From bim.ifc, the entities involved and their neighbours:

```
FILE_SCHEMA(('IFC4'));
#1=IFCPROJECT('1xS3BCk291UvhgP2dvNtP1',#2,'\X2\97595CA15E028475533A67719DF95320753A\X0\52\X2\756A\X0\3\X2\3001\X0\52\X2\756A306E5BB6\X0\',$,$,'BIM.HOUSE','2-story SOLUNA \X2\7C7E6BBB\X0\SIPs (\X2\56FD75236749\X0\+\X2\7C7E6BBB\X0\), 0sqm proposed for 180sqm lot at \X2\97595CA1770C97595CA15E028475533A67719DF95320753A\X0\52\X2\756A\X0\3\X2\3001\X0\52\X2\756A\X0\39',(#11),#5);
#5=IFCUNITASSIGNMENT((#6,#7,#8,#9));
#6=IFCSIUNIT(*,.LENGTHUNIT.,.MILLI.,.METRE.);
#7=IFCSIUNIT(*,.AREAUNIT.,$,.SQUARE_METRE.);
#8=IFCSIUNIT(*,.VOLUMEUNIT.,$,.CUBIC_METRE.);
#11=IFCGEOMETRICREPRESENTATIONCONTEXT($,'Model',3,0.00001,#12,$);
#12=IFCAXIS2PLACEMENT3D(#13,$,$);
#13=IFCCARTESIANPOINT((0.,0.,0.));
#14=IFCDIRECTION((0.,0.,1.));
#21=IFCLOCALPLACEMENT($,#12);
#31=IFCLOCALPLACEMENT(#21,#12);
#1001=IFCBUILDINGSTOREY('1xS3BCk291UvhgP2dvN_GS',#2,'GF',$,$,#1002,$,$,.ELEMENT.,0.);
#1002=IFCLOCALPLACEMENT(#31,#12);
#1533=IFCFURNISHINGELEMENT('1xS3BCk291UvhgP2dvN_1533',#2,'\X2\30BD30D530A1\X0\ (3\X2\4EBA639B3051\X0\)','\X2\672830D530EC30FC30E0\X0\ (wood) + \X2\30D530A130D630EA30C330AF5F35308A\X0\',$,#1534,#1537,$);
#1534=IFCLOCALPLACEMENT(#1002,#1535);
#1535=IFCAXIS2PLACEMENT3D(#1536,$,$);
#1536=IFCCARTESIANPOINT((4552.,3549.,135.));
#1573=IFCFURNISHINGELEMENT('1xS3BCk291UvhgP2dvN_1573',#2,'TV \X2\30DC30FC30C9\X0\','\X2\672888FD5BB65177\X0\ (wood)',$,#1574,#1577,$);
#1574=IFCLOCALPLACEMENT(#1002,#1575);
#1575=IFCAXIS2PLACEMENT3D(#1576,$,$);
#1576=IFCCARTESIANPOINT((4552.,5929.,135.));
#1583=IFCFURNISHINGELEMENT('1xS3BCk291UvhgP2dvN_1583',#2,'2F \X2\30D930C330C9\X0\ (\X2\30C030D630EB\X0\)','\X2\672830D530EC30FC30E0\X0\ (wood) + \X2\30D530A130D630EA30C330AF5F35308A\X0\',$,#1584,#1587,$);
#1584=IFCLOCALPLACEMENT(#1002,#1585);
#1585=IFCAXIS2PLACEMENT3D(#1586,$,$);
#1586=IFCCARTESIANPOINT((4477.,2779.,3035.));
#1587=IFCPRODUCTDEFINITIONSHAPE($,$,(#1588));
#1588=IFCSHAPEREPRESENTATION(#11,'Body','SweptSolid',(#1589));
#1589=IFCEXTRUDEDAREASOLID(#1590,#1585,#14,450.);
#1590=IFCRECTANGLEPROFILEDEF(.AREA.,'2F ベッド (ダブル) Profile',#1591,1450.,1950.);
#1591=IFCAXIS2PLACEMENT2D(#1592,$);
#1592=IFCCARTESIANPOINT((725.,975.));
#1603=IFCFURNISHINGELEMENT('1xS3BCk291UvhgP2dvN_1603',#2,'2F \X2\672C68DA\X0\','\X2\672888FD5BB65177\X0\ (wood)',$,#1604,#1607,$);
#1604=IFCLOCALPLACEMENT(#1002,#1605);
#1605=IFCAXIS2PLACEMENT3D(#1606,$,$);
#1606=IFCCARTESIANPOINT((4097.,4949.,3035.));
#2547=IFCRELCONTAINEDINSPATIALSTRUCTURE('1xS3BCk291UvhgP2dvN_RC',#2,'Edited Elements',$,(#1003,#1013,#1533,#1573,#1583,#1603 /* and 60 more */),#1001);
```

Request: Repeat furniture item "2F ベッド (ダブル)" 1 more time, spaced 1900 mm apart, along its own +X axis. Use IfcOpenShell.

```python
import ifcopenshell
import ifcopenshell.api.geometry
import ifcopenshell.api.root
import ifcopenshell.util.element
import ifcopenshell.util.placement

model = ifcopenshell.open("bim.ifc")


def reuse_history(source, copy):
    """copy_class also copies each property set's owner history, people and application; keep the originals."""
    for rel in copy.IsDefinedBy:
        if rel.is_a("IfcRelDefinesByProperties") and (history := rel.RelatingPropertyDefinition.OwnerHistory):
            rel.RelatingPropertyDefinition.OwnerHistory = source.OwnerHistory
            ifcopenshell.util.element.remove_deep2(model, history)


source = model.by_guid("1xS3BCk291UvhgP2dvN_1583")
base = ifcopenshell.util.placement.get_local_placement(source.ObjectPlacement)
step = base[:3, 0] * 1900.0

for i in range(1, 2):
    copy = ifcopenshell.api.root.copy_class(model, product=source)
    copy.Representation = ifcopenshell.util.element.copy_deep(
        model, source.Representation, exclude=["IfcGeometricRepresentationContext", "IfcRepresentationMap"]
    )
    reuse_history(source, copy)
    matrix = base.copy()
    matrix[:3, 3] += i * step
    print("added at", matrix[:3, 3].round(3) + 0.0)
    ifcopenshell.api.geometry.edit_object_placement(model, product=copy, matrix=matrix, is_si=False)

model.write("bim_updated.ifc")
```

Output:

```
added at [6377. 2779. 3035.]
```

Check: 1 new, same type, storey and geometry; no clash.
